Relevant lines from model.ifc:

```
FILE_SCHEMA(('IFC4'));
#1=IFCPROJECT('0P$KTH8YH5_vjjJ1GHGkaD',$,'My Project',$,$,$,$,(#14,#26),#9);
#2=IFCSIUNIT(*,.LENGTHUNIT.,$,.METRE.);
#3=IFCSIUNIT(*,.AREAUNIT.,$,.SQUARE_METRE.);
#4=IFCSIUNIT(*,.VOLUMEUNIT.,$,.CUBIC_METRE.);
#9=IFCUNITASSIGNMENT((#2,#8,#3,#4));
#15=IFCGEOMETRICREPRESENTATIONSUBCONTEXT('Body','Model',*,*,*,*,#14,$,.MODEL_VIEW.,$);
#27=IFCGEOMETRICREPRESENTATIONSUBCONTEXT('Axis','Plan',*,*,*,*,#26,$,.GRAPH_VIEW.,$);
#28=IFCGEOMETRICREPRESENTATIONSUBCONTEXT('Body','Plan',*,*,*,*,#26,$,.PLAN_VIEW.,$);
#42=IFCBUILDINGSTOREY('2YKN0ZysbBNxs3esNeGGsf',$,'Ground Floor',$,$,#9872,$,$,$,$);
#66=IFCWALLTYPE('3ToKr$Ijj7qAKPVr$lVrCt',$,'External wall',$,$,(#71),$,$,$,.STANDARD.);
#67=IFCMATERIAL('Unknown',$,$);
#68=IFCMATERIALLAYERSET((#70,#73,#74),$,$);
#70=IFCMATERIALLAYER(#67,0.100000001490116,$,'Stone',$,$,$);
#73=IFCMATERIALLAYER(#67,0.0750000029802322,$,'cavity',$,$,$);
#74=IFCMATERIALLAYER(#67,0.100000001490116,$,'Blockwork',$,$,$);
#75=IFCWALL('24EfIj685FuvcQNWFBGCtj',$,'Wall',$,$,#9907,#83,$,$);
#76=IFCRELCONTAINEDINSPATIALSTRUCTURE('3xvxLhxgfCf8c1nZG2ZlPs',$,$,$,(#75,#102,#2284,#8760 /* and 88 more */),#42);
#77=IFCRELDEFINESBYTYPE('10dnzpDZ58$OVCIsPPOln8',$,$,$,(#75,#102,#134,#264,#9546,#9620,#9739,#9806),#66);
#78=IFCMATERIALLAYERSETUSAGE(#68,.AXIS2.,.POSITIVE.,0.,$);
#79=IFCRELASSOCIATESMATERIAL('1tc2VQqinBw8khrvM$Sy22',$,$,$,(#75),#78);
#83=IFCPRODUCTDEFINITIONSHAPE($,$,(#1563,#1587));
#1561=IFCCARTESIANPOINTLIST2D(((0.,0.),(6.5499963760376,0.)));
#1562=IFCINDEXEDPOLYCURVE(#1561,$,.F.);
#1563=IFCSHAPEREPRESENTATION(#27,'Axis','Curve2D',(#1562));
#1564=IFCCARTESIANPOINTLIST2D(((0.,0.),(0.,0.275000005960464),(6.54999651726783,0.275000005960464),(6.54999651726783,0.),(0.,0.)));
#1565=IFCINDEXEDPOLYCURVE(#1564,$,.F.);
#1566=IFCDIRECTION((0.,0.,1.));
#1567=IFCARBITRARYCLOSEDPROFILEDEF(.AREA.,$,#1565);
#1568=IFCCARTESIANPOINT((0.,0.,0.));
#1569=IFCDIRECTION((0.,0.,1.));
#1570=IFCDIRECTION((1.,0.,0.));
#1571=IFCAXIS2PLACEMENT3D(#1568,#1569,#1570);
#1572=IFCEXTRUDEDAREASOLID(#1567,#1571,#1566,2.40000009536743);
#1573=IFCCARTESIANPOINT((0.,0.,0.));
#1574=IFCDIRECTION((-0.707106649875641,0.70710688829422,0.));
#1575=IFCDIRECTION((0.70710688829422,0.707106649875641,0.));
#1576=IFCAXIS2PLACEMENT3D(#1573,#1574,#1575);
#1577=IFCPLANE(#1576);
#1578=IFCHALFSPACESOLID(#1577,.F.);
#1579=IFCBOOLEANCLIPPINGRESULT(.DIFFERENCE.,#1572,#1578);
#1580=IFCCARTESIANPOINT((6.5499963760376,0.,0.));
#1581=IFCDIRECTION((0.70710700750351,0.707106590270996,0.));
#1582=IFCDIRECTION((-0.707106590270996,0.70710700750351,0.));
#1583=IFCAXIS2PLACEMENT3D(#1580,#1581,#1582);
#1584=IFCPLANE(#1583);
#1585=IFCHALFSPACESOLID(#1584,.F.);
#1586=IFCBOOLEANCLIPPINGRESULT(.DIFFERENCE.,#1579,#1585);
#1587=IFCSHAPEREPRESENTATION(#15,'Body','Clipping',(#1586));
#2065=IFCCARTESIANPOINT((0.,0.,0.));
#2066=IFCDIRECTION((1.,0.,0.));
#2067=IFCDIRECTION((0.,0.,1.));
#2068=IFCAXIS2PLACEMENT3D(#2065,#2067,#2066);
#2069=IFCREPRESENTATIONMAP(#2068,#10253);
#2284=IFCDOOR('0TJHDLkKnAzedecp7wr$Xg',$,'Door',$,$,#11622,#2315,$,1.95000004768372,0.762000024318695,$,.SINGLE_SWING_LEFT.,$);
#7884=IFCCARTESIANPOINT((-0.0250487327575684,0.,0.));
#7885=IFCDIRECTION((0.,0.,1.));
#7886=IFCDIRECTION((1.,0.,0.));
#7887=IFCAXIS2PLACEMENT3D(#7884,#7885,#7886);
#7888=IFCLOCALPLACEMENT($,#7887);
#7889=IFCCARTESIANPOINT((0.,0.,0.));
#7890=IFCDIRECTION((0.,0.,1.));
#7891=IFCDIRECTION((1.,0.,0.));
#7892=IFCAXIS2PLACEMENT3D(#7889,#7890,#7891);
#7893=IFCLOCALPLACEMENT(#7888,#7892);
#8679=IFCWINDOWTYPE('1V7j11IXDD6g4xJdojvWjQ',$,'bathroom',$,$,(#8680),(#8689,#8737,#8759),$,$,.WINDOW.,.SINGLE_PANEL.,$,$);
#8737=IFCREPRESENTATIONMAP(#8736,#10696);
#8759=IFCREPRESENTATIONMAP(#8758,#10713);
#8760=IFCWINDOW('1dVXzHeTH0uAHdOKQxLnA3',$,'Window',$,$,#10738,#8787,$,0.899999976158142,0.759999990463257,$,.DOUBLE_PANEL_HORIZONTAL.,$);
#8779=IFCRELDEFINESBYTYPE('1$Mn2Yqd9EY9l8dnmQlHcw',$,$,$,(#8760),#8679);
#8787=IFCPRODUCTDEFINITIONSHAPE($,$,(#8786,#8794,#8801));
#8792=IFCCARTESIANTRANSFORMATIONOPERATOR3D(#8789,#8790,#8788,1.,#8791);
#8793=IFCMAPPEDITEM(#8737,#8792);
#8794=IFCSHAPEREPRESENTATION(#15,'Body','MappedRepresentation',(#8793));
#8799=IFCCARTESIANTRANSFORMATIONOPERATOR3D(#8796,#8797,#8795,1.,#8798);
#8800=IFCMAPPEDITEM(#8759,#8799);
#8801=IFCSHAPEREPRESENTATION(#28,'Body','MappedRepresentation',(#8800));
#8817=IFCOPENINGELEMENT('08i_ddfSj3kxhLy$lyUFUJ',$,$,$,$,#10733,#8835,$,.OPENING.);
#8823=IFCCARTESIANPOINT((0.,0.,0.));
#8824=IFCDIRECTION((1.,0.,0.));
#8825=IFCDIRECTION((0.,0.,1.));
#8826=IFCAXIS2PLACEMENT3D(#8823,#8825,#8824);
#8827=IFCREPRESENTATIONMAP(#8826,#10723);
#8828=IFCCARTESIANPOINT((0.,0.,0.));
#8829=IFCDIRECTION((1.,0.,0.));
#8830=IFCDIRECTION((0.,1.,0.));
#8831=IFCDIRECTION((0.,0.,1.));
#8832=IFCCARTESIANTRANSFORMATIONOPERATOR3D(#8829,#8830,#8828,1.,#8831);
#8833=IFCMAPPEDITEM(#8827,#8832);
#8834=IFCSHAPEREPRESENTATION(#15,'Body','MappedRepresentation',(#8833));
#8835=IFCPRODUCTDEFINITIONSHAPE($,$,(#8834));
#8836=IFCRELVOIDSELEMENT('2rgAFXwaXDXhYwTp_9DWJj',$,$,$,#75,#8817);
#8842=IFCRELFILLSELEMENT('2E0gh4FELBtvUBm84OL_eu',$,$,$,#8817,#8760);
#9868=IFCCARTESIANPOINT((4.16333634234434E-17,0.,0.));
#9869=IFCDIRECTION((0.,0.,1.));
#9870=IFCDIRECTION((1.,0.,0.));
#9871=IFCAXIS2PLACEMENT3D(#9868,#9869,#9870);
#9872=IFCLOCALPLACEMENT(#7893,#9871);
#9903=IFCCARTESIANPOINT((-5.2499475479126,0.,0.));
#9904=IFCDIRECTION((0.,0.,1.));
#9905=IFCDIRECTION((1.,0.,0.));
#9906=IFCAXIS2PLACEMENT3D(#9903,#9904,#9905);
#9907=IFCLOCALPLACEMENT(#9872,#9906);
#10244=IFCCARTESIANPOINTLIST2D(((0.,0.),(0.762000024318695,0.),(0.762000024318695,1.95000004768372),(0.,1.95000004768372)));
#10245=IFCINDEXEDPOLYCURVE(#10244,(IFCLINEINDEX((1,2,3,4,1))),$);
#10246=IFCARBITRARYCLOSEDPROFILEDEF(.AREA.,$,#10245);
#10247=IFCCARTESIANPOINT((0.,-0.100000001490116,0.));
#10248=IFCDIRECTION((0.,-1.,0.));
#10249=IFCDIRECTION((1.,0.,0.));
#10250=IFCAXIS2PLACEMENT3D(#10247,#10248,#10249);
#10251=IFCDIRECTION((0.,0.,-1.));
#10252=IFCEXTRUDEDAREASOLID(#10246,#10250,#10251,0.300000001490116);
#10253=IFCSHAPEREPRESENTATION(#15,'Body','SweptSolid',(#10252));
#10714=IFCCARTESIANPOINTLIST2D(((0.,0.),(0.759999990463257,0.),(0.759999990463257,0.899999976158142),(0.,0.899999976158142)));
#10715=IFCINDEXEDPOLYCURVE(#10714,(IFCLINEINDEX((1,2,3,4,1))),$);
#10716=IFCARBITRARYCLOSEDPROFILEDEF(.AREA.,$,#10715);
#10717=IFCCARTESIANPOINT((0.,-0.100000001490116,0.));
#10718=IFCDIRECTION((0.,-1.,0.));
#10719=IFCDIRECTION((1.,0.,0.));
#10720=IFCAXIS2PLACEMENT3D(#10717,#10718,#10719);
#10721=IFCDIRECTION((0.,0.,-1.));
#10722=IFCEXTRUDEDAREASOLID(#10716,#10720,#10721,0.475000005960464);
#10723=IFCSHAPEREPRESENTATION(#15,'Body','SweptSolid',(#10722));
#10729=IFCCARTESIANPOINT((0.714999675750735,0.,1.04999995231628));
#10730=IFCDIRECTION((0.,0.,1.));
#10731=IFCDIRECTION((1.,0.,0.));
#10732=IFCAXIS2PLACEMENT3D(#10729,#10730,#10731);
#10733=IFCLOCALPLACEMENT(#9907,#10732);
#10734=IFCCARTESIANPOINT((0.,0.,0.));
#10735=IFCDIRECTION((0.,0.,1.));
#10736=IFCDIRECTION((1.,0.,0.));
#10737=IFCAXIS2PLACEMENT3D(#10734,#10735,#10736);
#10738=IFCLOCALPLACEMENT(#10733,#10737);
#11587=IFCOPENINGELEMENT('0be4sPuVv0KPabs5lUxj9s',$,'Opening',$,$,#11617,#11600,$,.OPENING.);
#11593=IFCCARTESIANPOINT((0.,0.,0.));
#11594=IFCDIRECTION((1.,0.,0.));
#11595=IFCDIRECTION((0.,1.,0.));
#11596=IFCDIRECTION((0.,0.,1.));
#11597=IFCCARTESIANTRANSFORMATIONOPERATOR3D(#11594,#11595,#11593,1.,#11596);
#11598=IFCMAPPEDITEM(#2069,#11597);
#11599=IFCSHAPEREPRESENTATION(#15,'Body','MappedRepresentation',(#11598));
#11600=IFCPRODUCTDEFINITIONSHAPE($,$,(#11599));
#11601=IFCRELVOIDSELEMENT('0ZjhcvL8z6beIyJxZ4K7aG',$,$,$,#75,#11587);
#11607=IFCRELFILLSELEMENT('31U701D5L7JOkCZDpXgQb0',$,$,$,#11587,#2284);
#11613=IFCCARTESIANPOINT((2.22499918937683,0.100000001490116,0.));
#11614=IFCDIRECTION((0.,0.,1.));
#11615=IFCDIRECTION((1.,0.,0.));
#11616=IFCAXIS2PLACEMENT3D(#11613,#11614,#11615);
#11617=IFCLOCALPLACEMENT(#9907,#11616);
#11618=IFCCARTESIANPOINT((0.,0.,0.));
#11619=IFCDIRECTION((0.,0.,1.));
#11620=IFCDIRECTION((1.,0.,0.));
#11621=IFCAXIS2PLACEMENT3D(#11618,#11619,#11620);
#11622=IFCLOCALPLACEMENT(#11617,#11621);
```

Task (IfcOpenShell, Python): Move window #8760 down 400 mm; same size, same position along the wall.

```python
import numpy as np
import ifcopenshell
import ifcopenshell.api.geometry
import ifcopenshell.util.placement
import ifcopenshell.util.unit

model = ifcopenshell.open("model.ifc")
unit_scale = ifcopenshell.util.unit.calculate_unit_scale(model)

window = model.by_guid("1dVXzHeTH0uAHdOKQxLnA3")
opening = window.FillsVoids[0].RelatingOpeningElement
dz = -0.4

shift = np.array([0.0, 0.0, dz])
# The window is placed relative to its opening, so it follows when the opening moves.
matrix = ifcopenshell.util.placement.get_local_placement(opening.ObjectPlacement)
matrix[:3, 3] += shift
ifcopenshell.api.geometry.edit_object_placement(
    model, product=opening, matrix=matrix, is_si=False, should_transform_children=True
)

print(f"moved by {dz * unit_scale:+.3f} m")

model.write("model_updated.ifc")
```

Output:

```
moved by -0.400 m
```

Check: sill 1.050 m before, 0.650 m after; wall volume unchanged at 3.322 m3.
